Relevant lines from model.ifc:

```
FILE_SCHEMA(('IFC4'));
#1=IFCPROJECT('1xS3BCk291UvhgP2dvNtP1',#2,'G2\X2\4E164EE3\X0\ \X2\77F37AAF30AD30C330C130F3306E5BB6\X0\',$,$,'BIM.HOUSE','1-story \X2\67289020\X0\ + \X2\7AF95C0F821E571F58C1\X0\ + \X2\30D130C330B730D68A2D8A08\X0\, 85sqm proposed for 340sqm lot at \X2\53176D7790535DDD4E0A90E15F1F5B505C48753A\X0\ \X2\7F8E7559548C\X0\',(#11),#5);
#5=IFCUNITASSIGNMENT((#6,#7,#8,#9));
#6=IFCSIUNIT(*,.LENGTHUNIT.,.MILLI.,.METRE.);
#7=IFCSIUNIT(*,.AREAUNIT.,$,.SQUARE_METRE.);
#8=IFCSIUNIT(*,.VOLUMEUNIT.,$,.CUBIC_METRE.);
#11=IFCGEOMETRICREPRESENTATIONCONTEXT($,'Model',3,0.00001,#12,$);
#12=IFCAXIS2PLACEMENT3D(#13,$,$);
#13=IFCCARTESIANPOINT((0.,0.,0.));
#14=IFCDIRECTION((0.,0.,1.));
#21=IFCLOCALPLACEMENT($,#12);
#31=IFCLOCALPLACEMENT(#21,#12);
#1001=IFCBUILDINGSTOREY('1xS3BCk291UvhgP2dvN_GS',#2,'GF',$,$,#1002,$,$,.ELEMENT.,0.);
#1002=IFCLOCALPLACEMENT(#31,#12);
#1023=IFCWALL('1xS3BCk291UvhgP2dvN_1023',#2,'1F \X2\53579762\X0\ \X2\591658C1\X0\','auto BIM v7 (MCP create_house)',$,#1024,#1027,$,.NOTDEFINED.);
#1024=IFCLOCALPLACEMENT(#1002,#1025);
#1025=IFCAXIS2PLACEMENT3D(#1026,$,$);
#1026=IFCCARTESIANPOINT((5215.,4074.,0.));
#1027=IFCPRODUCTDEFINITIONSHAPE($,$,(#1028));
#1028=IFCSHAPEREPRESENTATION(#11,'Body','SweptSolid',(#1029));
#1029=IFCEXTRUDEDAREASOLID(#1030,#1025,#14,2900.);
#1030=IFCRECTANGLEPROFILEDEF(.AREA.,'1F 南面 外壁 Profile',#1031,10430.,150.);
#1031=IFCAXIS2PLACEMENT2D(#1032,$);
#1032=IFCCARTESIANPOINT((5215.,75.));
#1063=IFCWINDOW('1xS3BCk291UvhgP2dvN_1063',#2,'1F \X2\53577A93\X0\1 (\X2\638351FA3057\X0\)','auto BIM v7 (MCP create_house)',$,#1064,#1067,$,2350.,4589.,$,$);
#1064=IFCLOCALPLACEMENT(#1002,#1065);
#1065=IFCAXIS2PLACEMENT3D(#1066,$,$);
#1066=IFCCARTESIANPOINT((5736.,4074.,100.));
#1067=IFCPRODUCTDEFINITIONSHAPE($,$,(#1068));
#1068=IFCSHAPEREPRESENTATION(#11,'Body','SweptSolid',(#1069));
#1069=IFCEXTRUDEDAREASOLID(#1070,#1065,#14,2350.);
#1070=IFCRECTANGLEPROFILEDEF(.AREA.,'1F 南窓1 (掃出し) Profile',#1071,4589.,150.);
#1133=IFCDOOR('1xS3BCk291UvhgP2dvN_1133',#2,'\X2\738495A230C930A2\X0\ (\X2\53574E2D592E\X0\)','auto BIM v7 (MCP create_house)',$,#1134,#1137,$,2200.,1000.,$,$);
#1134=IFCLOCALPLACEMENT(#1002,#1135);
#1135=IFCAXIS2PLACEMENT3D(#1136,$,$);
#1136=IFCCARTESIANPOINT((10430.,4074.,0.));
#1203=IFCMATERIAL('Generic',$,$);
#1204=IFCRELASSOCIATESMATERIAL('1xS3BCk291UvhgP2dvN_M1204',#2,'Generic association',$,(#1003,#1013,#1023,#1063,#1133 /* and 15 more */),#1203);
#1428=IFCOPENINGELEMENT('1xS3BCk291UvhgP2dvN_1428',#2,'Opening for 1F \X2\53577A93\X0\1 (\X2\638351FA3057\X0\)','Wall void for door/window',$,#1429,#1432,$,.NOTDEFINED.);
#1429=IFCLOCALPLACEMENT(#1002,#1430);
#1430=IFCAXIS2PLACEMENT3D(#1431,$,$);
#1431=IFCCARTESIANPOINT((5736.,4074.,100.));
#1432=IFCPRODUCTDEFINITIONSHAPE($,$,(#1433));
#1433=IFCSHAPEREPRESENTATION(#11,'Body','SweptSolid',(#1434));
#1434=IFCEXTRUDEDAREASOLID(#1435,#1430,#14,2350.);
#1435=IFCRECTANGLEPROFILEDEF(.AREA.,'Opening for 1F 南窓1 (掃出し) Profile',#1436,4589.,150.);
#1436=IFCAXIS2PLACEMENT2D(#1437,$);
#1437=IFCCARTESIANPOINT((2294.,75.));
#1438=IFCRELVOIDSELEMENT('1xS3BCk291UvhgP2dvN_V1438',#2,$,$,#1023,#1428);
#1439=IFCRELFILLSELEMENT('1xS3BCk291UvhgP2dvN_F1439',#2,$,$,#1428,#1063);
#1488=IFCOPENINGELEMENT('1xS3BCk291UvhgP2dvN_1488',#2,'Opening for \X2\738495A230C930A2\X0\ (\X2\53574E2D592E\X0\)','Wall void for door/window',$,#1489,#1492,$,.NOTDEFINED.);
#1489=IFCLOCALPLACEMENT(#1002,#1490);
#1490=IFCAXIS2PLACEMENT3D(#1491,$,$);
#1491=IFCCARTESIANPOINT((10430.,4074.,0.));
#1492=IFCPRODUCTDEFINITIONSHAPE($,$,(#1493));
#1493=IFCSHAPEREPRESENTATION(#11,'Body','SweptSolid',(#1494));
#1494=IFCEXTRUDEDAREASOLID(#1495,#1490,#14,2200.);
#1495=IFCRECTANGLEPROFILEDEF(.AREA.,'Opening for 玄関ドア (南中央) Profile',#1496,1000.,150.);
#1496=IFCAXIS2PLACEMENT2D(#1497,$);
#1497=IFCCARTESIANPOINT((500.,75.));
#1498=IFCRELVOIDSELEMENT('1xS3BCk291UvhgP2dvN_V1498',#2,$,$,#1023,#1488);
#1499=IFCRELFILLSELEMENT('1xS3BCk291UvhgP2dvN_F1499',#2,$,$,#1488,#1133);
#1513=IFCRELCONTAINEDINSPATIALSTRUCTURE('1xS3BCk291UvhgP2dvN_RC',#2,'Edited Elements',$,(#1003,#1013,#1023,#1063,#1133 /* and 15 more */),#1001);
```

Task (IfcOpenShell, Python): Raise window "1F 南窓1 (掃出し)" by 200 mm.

```python
import numpy as np
import ifcopenshell
import ifcopenshell.api.geometry
import ifcopenshell.util.placement
import ifcopenshell.util.unit

model = ifcopenshell.open("model.ifc")
unit_scale = ifcopenshell.util.unit.calculate_unit_scale(model)

window = model.by_guid("1xS3BCk291UvhgP2dvN_1063")
opening = window.FillsVoids[0].RelatingOpeningElement
dz = 200.0

shift = np.array([0.0, 0.0, dz])
# The window is not placed relative to its opening, so move both.
for product in (opening, window):
    matrix = ifcopenshell.util.placement.get_local_placement(product.ObjectPlacement)
    matrix[:3, 3] += shift
    ifcopenshell.api.geometry.edit_object_placement(model, product=product, matrix=matrix, is_si=False)

print(f"moved by {dz * unit_scale:+.3f} m")

model.write("model_edited.ifc")
```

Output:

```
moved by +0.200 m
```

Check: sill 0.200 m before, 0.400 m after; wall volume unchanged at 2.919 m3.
